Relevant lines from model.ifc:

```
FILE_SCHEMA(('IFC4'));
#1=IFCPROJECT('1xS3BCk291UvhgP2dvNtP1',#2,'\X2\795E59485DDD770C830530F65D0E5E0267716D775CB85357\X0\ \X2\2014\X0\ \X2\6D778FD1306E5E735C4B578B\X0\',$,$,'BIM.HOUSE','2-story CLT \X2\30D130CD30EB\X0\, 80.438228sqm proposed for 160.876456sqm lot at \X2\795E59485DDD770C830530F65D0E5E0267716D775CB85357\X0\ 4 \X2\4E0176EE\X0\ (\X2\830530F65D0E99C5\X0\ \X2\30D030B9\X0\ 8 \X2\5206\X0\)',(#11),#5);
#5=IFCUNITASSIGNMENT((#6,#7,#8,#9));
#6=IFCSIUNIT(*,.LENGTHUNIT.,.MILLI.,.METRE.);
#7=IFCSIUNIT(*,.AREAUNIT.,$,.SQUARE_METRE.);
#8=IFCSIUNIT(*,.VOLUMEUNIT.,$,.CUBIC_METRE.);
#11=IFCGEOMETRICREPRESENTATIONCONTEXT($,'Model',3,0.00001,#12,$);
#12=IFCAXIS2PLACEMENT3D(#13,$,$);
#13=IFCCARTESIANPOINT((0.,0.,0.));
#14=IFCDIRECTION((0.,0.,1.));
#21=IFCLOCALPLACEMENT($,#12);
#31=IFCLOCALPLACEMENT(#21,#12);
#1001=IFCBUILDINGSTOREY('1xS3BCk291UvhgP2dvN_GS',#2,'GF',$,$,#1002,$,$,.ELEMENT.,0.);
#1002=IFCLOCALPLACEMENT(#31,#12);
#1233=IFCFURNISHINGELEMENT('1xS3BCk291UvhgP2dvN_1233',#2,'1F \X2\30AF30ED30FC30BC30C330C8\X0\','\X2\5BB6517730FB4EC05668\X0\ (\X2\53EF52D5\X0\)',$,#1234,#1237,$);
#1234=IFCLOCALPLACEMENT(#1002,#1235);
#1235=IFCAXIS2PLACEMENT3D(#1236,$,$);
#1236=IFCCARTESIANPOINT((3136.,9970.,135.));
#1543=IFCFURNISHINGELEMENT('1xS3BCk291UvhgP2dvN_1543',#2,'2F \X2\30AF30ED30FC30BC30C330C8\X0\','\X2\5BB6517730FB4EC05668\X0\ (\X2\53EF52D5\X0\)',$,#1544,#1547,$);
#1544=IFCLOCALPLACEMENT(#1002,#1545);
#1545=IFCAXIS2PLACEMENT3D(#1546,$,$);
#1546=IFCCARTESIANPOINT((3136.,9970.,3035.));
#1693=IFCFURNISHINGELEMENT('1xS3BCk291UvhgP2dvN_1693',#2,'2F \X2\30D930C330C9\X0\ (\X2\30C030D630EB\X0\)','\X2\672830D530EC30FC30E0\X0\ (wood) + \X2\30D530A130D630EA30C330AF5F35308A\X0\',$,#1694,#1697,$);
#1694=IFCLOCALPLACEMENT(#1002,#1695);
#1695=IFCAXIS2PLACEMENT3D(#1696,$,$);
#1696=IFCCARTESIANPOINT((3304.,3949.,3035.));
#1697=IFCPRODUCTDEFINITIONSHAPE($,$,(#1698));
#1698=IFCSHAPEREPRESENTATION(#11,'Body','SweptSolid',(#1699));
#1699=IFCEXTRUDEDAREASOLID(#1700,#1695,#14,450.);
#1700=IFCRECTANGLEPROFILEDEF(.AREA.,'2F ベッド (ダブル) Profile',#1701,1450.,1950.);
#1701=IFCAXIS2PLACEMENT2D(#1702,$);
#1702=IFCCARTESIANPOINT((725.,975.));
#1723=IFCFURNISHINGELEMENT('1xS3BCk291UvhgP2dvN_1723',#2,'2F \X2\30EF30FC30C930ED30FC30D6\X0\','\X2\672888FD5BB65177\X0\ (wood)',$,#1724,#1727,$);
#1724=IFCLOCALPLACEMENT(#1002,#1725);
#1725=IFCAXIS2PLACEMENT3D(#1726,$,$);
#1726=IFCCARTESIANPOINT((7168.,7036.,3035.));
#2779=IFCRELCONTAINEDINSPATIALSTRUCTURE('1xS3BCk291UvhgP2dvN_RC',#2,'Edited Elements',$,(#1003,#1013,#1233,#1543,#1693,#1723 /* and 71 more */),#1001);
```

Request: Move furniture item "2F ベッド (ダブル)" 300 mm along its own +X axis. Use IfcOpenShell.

```python
import ifcopenshell
import ifcopenshell.api.geometry
import ifcopenshell.util.placement

model = ifcopenshell.open("model.ifc")

item = model.by_guid("1xS3BCk291UvhgP2dvN_1693")
matrix = ifcopenshell.util.placement.get_local_placement(item.ObjectPlacement)
matrix[:3, 3] += matrix[:3, 0] * 300.0
ifcopenshell.api.geometry.edit_object_placement(model, product=item, matrix=matrix, is_si=False)

print(ifcopenshell.util.placement.get_local_placement(item.ObjectPlacement).round(3) + 0.0)

model.write("model_v2.ifc")
```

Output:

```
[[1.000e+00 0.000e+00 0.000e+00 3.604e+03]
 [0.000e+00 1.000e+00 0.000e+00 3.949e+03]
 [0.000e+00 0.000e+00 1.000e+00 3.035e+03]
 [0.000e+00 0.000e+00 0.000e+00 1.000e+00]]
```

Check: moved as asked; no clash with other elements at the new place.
